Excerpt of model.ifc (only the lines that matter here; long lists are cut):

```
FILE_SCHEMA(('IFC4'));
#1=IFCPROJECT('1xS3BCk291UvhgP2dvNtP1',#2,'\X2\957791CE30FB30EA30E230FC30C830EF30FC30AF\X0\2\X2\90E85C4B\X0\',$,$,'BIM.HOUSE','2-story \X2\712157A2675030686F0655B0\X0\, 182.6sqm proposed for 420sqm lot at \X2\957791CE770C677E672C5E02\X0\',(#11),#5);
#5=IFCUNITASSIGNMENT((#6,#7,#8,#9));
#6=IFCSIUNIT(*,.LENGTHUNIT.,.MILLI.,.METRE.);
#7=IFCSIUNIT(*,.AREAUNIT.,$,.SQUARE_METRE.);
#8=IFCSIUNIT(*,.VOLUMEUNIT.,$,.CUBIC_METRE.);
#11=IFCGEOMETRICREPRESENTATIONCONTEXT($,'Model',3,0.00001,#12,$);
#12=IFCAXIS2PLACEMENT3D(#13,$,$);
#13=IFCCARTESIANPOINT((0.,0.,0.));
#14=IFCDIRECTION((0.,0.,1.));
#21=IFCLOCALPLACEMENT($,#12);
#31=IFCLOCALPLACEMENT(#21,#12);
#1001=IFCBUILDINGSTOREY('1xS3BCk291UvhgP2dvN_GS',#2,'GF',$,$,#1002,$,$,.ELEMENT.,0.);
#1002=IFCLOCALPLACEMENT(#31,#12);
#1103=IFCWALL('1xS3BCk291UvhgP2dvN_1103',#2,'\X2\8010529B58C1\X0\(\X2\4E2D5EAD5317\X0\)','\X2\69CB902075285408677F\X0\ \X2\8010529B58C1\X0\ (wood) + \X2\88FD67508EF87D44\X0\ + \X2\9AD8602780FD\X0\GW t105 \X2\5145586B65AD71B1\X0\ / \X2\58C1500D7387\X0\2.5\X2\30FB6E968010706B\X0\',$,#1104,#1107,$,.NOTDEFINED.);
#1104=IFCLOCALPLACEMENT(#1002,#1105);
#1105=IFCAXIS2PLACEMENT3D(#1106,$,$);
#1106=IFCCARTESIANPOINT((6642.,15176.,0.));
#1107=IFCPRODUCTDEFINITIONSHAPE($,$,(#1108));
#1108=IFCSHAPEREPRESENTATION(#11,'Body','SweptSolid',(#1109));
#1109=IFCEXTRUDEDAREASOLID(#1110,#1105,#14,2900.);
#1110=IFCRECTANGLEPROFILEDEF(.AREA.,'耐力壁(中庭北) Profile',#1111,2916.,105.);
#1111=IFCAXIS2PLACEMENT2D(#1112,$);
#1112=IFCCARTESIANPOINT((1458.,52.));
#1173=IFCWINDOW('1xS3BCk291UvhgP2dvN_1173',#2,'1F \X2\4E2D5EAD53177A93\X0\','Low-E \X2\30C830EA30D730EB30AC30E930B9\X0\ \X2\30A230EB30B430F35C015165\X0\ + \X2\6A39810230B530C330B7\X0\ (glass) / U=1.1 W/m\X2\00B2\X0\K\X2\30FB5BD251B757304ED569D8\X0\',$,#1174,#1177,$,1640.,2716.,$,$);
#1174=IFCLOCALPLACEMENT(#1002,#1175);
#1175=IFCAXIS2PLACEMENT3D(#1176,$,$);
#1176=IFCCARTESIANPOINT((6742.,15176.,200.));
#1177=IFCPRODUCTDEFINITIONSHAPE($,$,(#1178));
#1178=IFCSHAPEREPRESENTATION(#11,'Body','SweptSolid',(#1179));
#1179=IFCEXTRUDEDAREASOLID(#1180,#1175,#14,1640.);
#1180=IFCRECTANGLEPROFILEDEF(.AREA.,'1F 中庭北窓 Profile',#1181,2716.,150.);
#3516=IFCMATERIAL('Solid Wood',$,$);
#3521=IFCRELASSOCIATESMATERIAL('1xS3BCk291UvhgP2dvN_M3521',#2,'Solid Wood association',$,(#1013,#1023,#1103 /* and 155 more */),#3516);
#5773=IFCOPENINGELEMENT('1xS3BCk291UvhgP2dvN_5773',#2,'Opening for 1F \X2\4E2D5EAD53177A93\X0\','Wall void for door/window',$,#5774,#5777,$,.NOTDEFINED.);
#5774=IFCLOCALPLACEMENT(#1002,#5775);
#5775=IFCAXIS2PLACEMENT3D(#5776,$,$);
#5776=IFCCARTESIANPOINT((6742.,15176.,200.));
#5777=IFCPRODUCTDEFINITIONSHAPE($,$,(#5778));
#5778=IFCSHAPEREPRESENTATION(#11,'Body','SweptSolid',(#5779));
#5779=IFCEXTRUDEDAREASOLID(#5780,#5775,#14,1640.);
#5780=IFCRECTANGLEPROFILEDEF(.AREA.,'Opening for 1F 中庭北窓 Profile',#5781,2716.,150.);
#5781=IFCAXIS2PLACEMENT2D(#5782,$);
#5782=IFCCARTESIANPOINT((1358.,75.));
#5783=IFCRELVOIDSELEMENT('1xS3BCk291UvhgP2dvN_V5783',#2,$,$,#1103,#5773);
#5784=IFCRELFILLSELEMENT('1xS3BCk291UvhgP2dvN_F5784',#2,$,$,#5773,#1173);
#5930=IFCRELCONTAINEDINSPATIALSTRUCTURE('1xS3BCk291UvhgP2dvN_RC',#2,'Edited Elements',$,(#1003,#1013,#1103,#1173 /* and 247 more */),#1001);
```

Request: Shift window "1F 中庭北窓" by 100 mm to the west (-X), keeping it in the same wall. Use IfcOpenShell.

```python
import ifcopenshell
import ifcopenshell.api.geometry
import ifcopenshell.util.placement
import ifcopenshell.util.unit

model = ifcopenshell.open("model.ifc")
unit_scale = ifcopenshell.util.unit.calculate_unit_scale(model)

window = model.by_guid("1xS3BCk291UvhgP2dvN_1173")
opening = window.FillsVoids[0].RelatingOpeningElement
wall = opening.VoidsElements[0].RelatingBuildingElement

wall_matrix = ifcopenshell.util.placement.get_local_placement(wall.ObjectPlacement)
shift = wall_matrix[:3, 0] * -0.1 / unit_scale
before = ifcopenshell.util.placement.get_local_placement(window.ObjectPlacement)[:3, 3].copy()

# The window is not placed relative to its opening, so move both.
for product in (opening, window):
    matrix = ifcopenshell.util.placement.get_local_placement(product.ObjectPlacement)
    matrix[:3, 3] += shift
    ifcopenshell.api.geometry.edit_object_placement(model, product=product, matrix=matrix, is_si=False)

after = ifcopenshell.util.placement.get_local_placement(window.ObjectPlacement)[:3, 3]
print("window moved by", (after - before).round(3) + 0.0)

model.write("model-out.ifc")
```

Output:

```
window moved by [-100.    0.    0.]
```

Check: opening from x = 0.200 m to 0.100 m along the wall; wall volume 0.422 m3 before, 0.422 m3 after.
